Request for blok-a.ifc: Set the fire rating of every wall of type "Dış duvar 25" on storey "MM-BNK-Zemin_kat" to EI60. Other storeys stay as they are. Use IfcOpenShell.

First a look at what the model holds.

```python
import ifcopenshell
import ifcopenshell.util.element

model = ifcopenshell.open("blok-a.ifc")
print(model.schema)
storey = next(s for s in model.by_type("IfcBuildingStorey") if s.Name == "MM-BNK-Zemin_kat")
walls = [e for e in ifcopenshell.util.element.get_decomposition(storey) if e.is_a("IfcWall")]
seen = {}
for e in walls:
    element_type = ifcopenshell.util.element.get_type(e)
    key = (element_type.Name if element_type != e and element_type else None, ifcopenshell.util.element.get_pset(e, "Pset_WallCommon", "FireRating"))
    seen[key] = seen.get(key, 0) + 1
for (name, value), count in sorted(seen.items(), key=str):
    print(count, "x", name, "|", value)
```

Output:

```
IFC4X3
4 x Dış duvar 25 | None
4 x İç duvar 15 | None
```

```python
import ifcopenshell
import ifcopenshell.api.pset
import ifcopenshell.util.element

model = ifcopenshell.open("blok-a.ifc")

storey = next(s for s in model.by_type("IfcBuildingStorey") if s.Name == "MM-BNK-Zemin_kat")
walls = [e for e in ifcopenshell.util.element.get_decomposition(storey) if e.is_a("IfcWall")]

count = 0
for e in walls:
    element_type = ifcopenshell.util.element.get_type(e)
    if element_type in (None, e) or element_type.Name != "Dış duvar 25":
        continue
    # add_pset returns the element's existing set when there is one.
    pset = ifcopenshell.api.pset.add_pset(model, product=e, name="Pset_WallCommon")
    ifcopenshell.api.pset.edit_pset(model, pset=pset, properties={"FireRating": "EI60"})
    count += 1

print(count, "walls updated")

model.write("blok-a_edited.ifc")
```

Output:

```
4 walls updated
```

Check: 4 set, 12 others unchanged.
